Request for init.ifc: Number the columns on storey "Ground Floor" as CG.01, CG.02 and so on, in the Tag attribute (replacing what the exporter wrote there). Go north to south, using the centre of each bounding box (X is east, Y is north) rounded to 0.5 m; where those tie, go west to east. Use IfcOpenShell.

First a look at what the model holds.

```python
import ifcopenshell
import ifcopenshell.util.element
import ifcopenshell.util.placement

model = ifcopenshell.open("init.ifc")
print(model.schema)
storey = next(s for s in model.by_type("IfcBuildingStorey") if s.Name == "Ground Floor")
columns = [e for e in ifcopenshell.util.element.get_decomposition(storey) if e.is_a("IfcColumn")]
for e in sorted(columns, key=lambda e: e.id()):
    origin = ifcopenshell.util.placement.get_local_placement(e.ObjectPlacement)[:3, 3]
    print(e.id(), e.Tag, e.Name, origin.round(2) + 0.0, sep=" | ")
```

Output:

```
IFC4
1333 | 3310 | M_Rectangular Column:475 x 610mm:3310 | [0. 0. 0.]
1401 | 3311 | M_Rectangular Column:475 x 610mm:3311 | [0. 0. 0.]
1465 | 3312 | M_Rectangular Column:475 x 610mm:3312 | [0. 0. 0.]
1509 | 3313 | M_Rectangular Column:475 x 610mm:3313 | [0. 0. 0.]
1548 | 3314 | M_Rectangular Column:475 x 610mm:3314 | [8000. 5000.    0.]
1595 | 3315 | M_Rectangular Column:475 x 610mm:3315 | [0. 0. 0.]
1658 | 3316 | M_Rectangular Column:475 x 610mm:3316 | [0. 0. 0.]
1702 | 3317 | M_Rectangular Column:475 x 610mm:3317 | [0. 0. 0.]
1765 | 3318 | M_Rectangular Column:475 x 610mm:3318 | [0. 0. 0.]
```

```python
import ifcopenshell
import ifcopenshell.geom
import ifcopenshell.util.element
import ifcopenshell.util.shape

model = ifcopenshell.open("init.ifc")
settings = ifcopenshell.geom.settings()
settings.set("use-world-coords", True)


def centre(element):
    shape = ifcopenshell.geom.create_shape(settings, element)
    return ifcopenshell.util.shape.get_bbox_centroid(shape.geometry)


storey = next(s for s in model.by_type("IfcBuildingStorey") if s.Name == "Ground Floor")
columns = [e for e in ifcopenshell.util.element.get_decomposition(storey) if e.is_a("IfcColumn")]

# Insertion points can sit at a corner or the storey origin, so sort by the geometry (in metres).
centres = {e: centre(e) for e in columns}
columns.sort(key=lambda e: (-round(centres[e][1] / 0.5), centres[e][0]))

for i, e in enumerate(columns, start=1):
    number = f"CG.{i:02d}"
    e.Tag = number
    print(e.id(), number)

model.write("init_edited.ifc")
```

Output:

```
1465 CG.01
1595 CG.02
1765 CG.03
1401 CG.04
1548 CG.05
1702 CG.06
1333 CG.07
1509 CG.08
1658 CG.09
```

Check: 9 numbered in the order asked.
